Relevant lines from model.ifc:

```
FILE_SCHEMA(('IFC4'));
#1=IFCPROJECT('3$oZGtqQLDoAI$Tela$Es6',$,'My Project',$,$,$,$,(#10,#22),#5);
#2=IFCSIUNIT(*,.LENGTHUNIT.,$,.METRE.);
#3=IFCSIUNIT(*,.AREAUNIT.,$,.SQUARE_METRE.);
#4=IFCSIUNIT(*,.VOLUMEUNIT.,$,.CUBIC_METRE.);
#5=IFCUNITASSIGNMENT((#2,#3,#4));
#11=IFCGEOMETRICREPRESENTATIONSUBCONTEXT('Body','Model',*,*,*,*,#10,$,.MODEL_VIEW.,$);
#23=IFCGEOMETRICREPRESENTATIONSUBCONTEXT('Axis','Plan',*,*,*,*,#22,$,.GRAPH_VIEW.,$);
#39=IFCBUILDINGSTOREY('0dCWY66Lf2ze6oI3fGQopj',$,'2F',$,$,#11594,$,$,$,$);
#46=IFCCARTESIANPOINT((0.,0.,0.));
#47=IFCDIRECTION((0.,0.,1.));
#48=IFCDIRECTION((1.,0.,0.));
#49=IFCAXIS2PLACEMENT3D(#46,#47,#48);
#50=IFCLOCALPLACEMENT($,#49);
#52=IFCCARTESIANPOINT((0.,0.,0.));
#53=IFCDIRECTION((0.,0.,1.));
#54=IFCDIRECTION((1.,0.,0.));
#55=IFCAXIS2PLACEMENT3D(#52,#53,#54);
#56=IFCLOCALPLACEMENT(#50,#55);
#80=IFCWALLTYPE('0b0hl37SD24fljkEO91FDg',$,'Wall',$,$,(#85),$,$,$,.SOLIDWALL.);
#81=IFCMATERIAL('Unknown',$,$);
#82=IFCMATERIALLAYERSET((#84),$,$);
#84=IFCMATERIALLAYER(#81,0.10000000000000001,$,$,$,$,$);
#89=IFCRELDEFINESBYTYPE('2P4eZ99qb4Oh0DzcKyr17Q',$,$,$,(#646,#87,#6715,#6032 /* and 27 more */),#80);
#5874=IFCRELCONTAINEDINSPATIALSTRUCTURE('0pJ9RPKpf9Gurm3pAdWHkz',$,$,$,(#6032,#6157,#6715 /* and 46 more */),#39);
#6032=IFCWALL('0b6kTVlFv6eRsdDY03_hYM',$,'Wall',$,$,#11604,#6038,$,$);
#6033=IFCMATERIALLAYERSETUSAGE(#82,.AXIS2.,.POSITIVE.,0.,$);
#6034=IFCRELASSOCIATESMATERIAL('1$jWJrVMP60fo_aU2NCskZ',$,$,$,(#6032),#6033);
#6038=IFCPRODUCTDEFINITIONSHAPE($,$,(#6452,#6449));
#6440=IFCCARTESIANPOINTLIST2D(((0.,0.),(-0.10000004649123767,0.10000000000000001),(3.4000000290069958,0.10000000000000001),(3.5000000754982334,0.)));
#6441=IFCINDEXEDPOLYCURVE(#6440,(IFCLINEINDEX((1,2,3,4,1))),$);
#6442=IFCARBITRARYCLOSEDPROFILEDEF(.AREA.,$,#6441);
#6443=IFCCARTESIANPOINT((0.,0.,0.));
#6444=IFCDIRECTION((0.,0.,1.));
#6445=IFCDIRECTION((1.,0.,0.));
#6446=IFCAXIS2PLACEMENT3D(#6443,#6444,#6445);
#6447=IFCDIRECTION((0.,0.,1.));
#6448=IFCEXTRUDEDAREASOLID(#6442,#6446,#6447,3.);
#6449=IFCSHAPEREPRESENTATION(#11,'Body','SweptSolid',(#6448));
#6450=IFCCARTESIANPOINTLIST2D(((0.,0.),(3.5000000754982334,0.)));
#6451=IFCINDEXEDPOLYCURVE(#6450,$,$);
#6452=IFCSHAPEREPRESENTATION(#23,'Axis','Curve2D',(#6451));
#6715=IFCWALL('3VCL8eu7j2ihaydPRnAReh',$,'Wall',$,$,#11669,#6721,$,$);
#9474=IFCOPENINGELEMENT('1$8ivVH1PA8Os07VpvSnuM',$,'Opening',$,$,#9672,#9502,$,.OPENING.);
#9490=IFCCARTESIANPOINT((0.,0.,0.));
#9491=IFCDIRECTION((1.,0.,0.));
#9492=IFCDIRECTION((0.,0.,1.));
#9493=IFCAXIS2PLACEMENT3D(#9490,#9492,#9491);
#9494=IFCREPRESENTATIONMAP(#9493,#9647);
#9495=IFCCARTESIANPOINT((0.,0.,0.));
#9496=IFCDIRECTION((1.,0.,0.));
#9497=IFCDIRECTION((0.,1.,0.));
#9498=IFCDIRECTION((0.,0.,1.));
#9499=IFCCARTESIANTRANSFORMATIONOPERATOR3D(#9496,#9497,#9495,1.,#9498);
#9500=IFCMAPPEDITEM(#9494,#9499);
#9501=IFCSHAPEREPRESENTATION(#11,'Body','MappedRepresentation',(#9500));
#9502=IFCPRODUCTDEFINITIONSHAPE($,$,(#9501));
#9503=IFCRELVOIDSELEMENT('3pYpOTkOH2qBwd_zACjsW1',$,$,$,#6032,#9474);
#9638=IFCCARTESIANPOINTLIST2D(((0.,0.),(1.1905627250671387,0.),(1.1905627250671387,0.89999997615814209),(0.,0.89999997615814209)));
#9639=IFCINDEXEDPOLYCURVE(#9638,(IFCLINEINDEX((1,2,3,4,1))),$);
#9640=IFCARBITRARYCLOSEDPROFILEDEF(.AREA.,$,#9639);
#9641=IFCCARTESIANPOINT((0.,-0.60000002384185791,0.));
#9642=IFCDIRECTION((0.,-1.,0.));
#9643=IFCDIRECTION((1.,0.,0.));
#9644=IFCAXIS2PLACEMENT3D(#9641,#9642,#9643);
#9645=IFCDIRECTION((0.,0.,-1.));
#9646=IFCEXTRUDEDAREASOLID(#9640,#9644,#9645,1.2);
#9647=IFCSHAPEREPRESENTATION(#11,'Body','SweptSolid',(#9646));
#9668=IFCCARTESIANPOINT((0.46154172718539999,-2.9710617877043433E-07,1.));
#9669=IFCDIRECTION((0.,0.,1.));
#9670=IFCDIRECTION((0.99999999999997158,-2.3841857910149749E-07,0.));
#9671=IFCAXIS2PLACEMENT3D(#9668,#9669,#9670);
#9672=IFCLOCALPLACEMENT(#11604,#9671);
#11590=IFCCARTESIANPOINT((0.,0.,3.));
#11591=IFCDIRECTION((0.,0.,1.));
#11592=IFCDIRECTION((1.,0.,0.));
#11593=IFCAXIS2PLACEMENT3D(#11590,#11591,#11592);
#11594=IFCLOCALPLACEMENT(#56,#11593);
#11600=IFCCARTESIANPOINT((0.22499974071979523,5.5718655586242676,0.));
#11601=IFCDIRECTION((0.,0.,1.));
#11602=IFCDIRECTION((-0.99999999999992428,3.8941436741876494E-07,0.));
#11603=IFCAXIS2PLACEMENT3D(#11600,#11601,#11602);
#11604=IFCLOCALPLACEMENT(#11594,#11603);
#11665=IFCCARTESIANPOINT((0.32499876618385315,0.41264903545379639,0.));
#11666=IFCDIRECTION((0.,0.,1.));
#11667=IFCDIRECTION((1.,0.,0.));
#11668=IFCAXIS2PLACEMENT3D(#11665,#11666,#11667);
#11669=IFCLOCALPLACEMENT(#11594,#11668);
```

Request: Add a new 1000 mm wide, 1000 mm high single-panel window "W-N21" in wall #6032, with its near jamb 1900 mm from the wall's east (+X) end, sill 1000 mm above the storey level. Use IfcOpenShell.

```python
import numpy as np
import ifcopenshell
import ifcopenshell.api.feature
import ifcopenshell.api.geometry
import ifcopenshell.api.root
import ifcopenshell.api.spatial
import ifcopenshell.geom
import ifcopenshell.util.element
import ifcopenshell.util.placement
import ifcopenshell.util.representation
import ifcopenshell.util.shape
import ifcopenshell.util.unit

model = ifcopenshell.open("model.ifc")
unit_scale = ifcopenshell.util.unit.calculate_unit_scale(model)
settings = ifcopenshell.geom.settings()


def volume(element):
    """Net volume in cubic metres, openings subtracted."""
    shape = ifcopenshell.geom.create_shape(settings, element)
    return ifcopenshell.util.shape.get_volume(shape.geometry)


wall = model.by_guid("0b6kTVlFv6eRsdDY03_hYM")
storey = ifcopenshell.util.element.get_container(wall, ifc_class="IfcBuildingStorey")
context = ifcopenshell.util.representation.get_context(model, "Model", "Body", "MODEL_VIEW")
before = volume(wall)

width, height, from_end, sill = 1, 1, 1.9, 1  # metres

# The wall runs along its own X axis, and the end named is its -X end.
wall_shape = ifcopenshell.geom.create_shape(settings, wall)
x, y, z = ifcopenshell.util.shape.get_vertices(wall_shape.geometry).T
start = x.min() + from_end
face, thickness = float(y.min()), float(y.max() - y.min())
wall_matrix = ifcopenshell.util.placement.get_local_placement(wall.ObjectPlacement)
level = ifcopenshell.util.placement.get_local_placement(storey.ObjectPlacement)[2, 3]


def in_wall(x, y):
    """Placement at x, y metres in the wall's axes, at sill height."""
    matrix = wall_matrix.copy()
    matrix[:, 3] = wall_matrix @ np.array([x / unit_scale, y / unit_scale, 0.0, 1.0])
    matrix[2, 3] = level + sill / unit_scale
    return matrix


# Opening: a box that overshoots both wall faces by 50 mm.
opening = ifcopenshell.api.root.create_entity(model, ifc_class="IfcOpeningElement", predefined_type="OPENING")
box = ifcopenshell.api.geometry.add_wall_representation(
    model, context=context, length=width, height=height, thickness=thickness + 0.1
)
ifcopenshell.api.geometry.assign_representation(model, product=opening, representation=box)
ifcopenshell.api.geometry.edit_object_placement(model, product=opening, matrix=in_wall(start, face - 0.05), is_si=False)
ifcopenshell.api.feature.add_feature(model, feature=opening, element=wall)

window = ifcopenshell.api.root.create_entity(model, ifc_class="IfcWindow", name="W-N21", predefined_type="WINDOW")
window.OverallWidth, window.OverallHeight = width / unit_scale, height / unit_scale
window.PartitioningType = "SINGLE_PANEL"
body = ifcopenshell.api.geometry.add_window_representation(
    model,
    context=context,
    overall_width=window.OverallWidth,
    overall_height=window.OverallHeight,
    partition_type="SINGLE_PANEL",
)
ifcopenshell.api.geometry.assign_representation(model, product=window, representation=body)
ifcopenshell.api.spatial.assign_container(model, products=[window], relating_structure=storey)
ifcopenshell.api.feature.add_filling(model, opening=opening, element=window)

# Centre the window in the wall's thickness.
ifcopenshell.api.geometry.edit_object_placement(model, product=window, matrix=in_wall(start, face), is_si=False)
window_shape = ifcopenshell.geom.create_shape(settings, window)
depth = ifcopenshell.util.shape.get_vertices(window_shape.geometry)[:, 1]
offset = face + thickness / 2 - (depth.min() + depth.max()) / 2
ifcopenshell.api.geometry.edit_object_placement(model, product=window, matrix=in_wall(start, offset), is_si=False)

after = volume(wall)

print(f"wall volume {before:.3f} -> {after:.3f} m3")

model.write("model_rev.ifc")
```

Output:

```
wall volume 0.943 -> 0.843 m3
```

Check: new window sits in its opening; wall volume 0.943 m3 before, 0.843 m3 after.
